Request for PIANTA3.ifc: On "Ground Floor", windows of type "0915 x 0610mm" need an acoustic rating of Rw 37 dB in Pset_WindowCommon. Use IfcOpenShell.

First a look at what the model holds.

```python
import ifcopenshell
import ifcopenshell.util.element

model = ifcopenshell.open("PIANTA3.ifc")
print(model.schema)
storey = next(s for s in model.by_type("IfcBuildingStorey") if s.Name == "Ground Floor")
windows = [e for e in ifcopenshell.util.element.get_decomposition(storey) if e.is_a("IfcWindow")]
seen = {}
for e in windows:
    element_type = ifcopenshell.util.element.get_type(e)
    key = (element_type.Name if element_type != e and element_type else None, ifcopenshell.util.element.get_pset(e, "Pset_WindowCommon", "AcousticRating"))
    seen[key] = seen.get(key, 0) + 1
for (name, value), count in sorted(seen.items(), key=str):
    print(count, "x", name, "|", value)
```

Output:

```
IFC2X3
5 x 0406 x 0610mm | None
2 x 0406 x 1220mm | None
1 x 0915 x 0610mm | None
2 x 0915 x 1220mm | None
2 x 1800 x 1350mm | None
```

```python
import ifcopenshell
import ifcopenshell.api.pset
import ifcopenshell.util.element

model = ifcopenshell.open("PIANTA3.ifc")

storey = next(s for s in model.by_type("IfcBuildingStorey") if s.Name == "Ground Floor")
windows = [e for e in ifcopenshell.util.element.get_decomposition(storey) if e.is_a("IfcWindow")]

count = 0
for e in windows:
    element_type = ifcopenshell.util.element.get_type(e)
    if element_type in (None, e) or element_type.Name != "0915 x 0610mm":
        continue
    # add_pset returns the element's existing set when there is one.
    pset = ifcopenshell.api.pset.add_pset(model, product=e, name="Pset_WindowCommon")
    ifcopenshell.api.pset.edit_pset(model, pset=pset, properties={"AcousticRating": "Rw 37 dB"})
    count += 1

print(count, "windows updated")

model.write("PIANTA3_rev.ifc")
```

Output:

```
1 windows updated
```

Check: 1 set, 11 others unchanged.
